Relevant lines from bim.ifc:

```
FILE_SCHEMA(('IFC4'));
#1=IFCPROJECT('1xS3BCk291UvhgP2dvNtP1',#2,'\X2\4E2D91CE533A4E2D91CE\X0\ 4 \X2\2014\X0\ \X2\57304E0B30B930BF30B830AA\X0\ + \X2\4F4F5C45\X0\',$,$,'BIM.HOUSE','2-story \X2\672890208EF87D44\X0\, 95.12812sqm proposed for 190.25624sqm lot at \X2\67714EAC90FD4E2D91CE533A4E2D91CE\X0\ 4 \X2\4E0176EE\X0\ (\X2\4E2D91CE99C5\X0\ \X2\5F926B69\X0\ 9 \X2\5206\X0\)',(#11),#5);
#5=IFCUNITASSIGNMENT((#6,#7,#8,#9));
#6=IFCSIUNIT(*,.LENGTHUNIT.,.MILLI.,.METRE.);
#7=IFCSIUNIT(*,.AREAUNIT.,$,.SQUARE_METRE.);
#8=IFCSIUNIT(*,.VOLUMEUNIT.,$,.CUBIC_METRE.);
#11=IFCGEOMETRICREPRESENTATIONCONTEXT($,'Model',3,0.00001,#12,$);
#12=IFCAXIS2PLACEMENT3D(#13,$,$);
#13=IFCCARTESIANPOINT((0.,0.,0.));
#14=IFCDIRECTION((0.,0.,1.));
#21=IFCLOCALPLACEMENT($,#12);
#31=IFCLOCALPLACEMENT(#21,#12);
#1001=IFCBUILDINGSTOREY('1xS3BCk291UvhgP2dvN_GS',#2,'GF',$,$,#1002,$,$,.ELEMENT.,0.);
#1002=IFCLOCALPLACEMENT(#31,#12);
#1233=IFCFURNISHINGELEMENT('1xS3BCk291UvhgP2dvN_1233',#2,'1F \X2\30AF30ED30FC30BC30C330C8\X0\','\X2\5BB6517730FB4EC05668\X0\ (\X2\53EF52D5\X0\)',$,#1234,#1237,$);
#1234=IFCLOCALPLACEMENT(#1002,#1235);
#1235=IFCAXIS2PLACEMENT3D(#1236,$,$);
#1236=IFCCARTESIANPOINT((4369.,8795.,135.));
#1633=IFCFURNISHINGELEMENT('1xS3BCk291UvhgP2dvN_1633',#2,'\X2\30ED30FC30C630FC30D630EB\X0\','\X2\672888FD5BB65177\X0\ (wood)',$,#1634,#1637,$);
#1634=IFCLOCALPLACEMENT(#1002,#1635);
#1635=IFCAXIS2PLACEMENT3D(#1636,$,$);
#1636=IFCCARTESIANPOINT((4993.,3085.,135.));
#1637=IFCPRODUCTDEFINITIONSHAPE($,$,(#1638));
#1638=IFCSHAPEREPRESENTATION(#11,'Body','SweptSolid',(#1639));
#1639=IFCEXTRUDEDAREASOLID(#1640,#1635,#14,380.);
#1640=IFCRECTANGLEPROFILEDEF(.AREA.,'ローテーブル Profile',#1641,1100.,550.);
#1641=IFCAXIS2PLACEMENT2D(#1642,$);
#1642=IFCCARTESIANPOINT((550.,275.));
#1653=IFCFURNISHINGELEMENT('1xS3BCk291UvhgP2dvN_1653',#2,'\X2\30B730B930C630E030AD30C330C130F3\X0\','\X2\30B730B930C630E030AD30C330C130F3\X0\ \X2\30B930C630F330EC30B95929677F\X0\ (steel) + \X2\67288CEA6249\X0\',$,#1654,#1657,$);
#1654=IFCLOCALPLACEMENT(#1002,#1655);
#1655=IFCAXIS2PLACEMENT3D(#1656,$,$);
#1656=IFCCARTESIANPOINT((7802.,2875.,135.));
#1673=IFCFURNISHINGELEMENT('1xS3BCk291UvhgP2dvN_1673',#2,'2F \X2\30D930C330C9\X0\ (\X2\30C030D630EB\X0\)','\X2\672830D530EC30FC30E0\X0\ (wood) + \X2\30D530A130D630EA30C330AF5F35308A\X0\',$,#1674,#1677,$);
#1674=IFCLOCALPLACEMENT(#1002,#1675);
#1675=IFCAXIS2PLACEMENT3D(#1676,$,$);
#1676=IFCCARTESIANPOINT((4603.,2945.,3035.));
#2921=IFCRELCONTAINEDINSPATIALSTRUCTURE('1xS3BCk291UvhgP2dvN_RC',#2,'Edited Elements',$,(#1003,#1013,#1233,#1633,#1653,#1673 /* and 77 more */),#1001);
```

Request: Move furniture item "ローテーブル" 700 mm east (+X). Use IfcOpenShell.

```python
import ifcopenshell
import ifcopenshell.api.geometry
import ifcopenshell.util.placement
import ifcopenshell.util.unit

model = ifcopenshell.open("bim.ifc")
unit_scale = ifcopenshell.util.unit.calculate_unit_scale(model)

item = model.by_guid("1xS3BCk291UvhgP2dvN_1633")
matrix = ifcopenshell.util.placement.get_local_placement(item.ObjectPlacement)
matrix[0, 3] += 0.7 / unit_scale
ifcopenshell.api.geometry.edit_object_placement(model, product=item, matrix=matrix, is_si=False)

print(ifcopenshell.util.placement.get_local_placement(item.ObjectPlacement).round(3) + 0.0)

model.write("bim_rev.ifc")
```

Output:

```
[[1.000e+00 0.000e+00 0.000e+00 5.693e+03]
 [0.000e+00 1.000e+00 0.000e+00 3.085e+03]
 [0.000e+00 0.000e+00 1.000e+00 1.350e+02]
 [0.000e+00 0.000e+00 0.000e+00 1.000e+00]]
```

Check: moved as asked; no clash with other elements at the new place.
